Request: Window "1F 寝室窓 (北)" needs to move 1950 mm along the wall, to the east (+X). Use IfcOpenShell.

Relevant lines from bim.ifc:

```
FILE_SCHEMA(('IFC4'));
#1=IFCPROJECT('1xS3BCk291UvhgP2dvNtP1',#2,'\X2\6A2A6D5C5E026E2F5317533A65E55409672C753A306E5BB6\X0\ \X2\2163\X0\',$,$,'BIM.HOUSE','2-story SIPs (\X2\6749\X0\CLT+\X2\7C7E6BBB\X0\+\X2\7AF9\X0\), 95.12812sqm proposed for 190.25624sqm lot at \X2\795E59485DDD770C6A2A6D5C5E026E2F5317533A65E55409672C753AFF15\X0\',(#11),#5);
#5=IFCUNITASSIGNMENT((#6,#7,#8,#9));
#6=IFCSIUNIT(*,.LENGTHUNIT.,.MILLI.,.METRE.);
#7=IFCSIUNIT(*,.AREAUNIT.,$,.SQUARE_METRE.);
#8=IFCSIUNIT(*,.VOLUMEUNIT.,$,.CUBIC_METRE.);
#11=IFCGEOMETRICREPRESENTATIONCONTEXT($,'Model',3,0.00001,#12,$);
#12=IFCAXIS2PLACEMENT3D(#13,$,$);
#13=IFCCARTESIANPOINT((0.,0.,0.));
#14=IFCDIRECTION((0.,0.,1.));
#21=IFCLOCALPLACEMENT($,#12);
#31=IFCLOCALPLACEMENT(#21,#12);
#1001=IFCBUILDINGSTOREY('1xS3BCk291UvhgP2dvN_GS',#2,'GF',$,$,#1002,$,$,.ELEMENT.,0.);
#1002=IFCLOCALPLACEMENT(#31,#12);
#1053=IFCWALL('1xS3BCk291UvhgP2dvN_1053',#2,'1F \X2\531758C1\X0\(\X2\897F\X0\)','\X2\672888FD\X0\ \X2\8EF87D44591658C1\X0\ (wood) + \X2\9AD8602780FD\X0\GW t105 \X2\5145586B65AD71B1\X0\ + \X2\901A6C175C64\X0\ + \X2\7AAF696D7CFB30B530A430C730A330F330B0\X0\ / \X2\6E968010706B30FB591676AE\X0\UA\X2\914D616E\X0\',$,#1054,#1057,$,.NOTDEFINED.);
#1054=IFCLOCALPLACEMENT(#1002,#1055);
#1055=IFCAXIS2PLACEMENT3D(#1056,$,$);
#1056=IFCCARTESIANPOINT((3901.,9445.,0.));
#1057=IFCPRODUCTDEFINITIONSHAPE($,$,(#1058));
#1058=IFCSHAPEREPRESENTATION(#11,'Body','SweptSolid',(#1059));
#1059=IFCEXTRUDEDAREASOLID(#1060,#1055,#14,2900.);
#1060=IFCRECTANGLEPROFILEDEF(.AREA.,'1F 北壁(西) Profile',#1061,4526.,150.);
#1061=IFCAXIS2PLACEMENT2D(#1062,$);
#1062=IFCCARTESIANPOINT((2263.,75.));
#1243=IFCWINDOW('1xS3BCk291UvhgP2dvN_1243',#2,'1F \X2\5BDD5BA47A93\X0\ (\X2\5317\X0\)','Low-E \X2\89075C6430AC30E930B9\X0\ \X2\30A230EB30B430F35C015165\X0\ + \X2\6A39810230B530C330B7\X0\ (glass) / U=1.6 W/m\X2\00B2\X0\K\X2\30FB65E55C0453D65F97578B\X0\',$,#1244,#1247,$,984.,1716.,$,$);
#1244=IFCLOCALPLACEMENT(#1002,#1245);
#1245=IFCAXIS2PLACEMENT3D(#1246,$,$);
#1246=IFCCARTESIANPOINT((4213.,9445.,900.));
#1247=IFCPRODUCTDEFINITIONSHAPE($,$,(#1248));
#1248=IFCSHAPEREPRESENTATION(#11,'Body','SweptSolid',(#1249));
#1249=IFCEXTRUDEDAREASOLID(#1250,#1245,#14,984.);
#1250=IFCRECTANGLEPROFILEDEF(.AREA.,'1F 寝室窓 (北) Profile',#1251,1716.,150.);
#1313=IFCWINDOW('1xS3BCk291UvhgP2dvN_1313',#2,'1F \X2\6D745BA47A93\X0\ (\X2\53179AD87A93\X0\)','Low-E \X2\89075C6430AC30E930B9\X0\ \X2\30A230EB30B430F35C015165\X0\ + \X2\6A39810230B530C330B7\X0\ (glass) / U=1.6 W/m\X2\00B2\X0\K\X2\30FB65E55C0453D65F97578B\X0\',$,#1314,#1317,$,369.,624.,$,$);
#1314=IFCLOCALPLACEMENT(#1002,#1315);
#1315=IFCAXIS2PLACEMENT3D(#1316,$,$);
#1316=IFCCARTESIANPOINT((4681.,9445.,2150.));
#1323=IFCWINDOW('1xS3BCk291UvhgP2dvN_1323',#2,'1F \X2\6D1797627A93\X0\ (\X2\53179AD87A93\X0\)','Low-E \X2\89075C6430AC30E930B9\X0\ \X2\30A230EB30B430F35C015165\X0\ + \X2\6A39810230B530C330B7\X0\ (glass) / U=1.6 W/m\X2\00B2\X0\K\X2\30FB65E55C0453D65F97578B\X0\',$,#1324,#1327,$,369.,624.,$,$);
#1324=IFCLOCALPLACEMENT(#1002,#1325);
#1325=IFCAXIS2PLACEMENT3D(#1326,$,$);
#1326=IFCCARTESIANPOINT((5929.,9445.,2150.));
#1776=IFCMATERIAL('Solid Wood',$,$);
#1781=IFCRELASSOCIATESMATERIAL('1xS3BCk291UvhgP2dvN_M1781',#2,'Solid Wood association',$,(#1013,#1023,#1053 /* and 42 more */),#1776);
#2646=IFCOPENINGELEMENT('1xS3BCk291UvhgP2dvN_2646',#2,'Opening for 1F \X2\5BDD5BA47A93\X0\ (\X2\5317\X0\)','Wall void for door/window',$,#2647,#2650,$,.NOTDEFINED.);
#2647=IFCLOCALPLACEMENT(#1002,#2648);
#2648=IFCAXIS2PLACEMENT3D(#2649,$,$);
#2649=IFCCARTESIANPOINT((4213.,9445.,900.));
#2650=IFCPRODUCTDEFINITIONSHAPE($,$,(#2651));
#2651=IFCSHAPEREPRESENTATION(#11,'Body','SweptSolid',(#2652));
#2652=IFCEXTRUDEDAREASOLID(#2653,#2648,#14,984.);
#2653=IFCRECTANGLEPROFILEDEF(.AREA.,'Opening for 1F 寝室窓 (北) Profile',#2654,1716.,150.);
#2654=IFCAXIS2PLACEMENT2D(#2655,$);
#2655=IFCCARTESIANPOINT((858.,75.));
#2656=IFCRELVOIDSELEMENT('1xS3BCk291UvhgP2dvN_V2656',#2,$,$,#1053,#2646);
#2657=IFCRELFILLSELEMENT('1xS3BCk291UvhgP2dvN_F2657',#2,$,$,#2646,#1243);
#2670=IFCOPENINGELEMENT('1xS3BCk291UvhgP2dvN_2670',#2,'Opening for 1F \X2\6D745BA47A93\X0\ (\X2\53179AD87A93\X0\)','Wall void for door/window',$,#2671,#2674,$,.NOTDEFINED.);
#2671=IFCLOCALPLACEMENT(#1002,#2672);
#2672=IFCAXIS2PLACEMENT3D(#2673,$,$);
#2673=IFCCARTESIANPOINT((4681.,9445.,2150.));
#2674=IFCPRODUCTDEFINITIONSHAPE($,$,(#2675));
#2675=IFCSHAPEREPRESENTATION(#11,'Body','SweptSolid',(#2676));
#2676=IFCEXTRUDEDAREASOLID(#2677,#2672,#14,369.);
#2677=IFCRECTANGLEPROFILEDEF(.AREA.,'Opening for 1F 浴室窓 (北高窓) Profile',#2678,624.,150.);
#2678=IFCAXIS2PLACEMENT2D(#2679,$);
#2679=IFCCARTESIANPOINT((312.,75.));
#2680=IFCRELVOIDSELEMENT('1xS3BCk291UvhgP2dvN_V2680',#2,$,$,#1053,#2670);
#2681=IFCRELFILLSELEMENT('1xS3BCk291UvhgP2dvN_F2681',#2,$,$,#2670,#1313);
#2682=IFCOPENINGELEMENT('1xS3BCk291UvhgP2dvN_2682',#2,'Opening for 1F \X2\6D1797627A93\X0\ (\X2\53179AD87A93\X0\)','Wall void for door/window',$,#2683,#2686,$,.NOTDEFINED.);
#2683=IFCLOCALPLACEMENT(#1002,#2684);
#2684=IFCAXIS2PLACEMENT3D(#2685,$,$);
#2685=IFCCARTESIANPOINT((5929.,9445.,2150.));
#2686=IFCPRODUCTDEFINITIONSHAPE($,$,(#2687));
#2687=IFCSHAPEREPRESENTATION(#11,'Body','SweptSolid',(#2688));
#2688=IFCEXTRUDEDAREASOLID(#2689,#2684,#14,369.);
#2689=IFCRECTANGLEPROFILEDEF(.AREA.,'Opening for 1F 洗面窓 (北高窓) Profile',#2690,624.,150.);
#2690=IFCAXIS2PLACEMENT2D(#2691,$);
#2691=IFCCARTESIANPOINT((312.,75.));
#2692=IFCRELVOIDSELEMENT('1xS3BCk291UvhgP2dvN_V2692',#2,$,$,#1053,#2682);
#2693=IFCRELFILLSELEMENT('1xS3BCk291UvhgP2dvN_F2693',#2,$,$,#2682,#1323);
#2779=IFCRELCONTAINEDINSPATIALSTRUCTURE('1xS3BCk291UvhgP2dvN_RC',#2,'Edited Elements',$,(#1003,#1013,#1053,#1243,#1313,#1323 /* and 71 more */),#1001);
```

```python
import ifcopenshell
import ifcopenshell.api.geometry
import ifcopenshell.util.placement
import ifcopenshell.util.unit

model = ifcopenshell.open("bim.ifc")
unit_scale = ifcopenshell.util.unit.calculate_unit_scale(model)

window = model.by_guid("1xS3BCk291UvhgP2dvN_1243")
opening = window.FillsVoids[0].RelatingOpeningElement
wall = opening.VoidsElements[0].RelatingBuildingElement

wall_matrix = ifcopenshell.util.placement.get_local_placement(wall.ObjectPlacement)
shift = wall_matrix[:3, 0] * 1.95 / unit_scale
before = ifcopenshell.util.placement.get_local_placement(window.ObjectPlacement)[:3, 3].copy()

# The window is not placed relative to its opening, so move both.
for product in (opening, window):
    matrix = ifcopenshell.util.placement.get_local_placement(product.ObjectPlacement)
    matrix[:3, 3] += shift
    ifcopenshell.api.geometry.edit_object_placement(model, product=product, matrix=matrix, is_si=False)

after = ifcopenshell.util.placement.get_local_placement(window.ObjectPlacement)[:3, 3]
print("window moved by", (after - before).round(3) + 0.0)

model.write("bim_rev.ifc")
```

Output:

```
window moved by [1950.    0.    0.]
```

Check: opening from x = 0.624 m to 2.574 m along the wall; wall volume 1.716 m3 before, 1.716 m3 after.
